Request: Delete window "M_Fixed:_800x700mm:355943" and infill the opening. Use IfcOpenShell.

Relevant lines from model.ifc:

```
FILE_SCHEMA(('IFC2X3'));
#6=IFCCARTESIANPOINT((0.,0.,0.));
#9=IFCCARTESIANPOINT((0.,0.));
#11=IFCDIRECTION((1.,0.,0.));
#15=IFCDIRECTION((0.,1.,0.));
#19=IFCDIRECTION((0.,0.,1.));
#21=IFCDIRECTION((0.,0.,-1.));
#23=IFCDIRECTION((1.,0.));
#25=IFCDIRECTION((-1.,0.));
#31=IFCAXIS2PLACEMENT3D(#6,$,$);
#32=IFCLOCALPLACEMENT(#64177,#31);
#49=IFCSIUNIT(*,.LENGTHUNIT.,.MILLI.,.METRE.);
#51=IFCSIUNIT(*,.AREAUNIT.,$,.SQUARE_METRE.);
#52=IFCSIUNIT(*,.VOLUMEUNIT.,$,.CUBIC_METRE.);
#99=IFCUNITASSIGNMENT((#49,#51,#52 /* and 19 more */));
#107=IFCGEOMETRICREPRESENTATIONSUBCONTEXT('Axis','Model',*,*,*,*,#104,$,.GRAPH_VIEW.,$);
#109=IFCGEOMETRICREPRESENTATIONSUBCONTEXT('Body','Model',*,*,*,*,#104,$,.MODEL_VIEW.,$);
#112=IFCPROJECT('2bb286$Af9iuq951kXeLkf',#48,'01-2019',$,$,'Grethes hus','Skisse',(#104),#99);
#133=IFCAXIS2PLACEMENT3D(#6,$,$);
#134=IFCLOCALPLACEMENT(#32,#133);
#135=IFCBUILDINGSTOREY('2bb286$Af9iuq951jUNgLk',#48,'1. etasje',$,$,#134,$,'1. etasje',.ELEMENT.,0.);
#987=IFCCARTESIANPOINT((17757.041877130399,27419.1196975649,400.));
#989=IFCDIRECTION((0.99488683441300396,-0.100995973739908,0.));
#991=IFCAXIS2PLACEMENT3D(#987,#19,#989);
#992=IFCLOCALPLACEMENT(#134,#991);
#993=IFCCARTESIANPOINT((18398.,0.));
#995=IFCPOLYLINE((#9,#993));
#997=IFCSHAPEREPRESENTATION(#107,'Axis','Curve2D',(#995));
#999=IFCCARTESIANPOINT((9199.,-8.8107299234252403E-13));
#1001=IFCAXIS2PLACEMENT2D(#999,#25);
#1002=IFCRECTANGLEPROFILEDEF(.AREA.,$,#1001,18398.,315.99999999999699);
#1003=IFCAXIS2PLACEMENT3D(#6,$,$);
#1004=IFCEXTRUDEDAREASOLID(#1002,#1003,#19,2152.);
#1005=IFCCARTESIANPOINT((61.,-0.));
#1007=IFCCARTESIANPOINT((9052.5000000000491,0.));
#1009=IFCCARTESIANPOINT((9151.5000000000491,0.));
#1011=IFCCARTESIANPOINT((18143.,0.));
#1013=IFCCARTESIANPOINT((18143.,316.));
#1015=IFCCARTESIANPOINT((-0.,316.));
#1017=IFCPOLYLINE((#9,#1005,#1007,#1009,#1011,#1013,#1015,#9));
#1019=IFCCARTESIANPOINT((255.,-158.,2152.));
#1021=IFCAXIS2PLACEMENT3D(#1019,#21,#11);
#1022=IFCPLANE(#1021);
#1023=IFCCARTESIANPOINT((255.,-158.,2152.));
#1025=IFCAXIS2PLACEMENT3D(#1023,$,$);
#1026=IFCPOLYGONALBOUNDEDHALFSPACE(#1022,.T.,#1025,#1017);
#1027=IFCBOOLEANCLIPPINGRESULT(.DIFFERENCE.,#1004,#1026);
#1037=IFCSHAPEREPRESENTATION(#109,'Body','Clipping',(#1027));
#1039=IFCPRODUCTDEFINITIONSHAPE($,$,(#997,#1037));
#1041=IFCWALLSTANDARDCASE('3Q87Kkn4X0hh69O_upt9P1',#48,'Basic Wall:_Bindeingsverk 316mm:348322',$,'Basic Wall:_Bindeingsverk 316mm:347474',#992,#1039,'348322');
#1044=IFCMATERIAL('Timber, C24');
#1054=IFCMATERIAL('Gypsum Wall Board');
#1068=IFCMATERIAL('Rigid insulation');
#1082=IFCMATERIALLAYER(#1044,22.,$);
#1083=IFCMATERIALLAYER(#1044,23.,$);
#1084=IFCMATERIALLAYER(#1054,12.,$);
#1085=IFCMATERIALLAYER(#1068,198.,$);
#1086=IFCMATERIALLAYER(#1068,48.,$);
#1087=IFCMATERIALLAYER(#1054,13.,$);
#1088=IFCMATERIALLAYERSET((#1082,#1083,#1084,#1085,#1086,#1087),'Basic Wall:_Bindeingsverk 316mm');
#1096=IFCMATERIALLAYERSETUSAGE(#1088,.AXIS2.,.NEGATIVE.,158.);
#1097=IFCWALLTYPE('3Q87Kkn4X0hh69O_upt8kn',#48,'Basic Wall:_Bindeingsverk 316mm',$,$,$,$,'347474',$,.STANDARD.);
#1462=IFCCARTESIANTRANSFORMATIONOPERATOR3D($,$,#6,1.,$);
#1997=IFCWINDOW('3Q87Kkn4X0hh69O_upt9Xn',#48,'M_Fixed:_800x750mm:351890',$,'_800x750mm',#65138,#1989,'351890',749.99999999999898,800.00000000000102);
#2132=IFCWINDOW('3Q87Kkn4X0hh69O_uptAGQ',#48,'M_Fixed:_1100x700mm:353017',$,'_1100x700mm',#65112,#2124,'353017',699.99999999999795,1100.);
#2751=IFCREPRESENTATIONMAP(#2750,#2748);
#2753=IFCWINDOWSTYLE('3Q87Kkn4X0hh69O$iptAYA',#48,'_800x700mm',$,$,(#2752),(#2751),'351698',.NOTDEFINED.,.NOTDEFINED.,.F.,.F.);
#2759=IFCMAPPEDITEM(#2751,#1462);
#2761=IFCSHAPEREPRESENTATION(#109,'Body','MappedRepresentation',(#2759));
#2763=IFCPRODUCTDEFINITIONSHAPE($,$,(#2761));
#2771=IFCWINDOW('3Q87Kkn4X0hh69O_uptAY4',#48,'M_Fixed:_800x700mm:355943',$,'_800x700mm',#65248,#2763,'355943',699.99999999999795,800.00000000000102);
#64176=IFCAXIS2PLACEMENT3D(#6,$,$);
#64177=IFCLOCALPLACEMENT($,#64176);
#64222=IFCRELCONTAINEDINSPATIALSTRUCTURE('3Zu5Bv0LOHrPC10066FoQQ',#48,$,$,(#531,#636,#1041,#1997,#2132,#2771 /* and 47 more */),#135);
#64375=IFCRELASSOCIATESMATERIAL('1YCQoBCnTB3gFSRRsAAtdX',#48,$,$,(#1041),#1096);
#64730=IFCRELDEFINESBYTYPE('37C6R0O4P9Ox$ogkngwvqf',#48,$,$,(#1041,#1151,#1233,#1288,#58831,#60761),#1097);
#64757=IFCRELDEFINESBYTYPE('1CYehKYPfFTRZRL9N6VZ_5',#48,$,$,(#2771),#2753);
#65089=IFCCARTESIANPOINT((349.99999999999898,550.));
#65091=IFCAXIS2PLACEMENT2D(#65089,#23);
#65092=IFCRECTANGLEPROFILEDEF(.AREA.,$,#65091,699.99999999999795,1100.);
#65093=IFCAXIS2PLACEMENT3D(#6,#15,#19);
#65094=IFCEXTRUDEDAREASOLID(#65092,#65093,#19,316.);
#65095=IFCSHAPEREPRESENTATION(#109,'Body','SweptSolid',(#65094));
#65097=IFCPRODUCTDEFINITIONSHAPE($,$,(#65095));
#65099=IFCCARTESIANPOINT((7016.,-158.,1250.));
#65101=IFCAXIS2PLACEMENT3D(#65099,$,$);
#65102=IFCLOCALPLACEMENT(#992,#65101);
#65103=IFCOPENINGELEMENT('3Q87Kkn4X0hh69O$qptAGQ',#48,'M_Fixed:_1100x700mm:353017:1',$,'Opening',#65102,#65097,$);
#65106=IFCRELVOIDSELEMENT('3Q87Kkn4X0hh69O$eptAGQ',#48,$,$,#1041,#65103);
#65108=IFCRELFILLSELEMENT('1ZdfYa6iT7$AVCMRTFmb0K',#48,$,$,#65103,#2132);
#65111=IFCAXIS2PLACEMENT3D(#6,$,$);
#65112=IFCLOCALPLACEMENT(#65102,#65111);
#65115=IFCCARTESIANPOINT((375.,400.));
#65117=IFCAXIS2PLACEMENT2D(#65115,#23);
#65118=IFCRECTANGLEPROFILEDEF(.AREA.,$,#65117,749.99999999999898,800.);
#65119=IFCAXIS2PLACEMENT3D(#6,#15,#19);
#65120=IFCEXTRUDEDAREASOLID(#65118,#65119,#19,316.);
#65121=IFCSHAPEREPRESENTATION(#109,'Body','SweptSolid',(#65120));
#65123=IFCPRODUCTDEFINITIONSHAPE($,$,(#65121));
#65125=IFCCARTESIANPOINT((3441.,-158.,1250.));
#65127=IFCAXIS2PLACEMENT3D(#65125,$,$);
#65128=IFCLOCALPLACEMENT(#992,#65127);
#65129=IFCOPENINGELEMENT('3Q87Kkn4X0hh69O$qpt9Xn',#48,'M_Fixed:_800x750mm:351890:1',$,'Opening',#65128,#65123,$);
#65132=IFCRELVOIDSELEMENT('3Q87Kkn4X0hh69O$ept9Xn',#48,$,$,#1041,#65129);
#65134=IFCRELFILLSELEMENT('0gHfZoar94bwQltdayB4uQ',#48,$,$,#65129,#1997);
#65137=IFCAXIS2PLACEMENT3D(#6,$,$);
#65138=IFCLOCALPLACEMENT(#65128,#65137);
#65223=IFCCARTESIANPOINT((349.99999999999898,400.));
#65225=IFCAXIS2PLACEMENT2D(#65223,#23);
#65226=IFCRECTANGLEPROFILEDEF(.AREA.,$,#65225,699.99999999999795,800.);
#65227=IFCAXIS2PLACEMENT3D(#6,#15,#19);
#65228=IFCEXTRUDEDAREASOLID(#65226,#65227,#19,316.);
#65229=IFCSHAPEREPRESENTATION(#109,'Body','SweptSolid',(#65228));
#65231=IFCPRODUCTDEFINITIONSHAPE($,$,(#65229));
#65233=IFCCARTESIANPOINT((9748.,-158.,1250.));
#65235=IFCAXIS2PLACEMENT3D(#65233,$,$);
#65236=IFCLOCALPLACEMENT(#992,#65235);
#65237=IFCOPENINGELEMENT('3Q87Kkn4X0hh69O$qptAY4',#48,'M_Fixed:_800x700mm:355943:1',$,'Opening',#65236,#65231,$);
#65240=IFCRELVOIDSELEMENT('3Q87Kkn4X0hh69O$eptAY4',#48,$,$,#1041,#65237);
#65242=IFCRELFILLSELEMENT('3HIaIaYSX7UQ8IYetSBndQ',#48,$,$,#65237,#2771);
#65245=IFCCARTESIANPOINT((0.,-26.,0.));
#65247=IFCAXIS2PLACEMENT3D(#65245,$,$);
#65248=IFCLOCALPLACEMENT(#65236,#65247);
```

```python
import ifcopenshell
import ifcopenshell.api.feature
import ifcopenshell.api.root
import ifcopenshell.geom
import ifcopenshell.util.shape

model = ifcopenshell.open("model.ifc")
settings = ifcopenshell.geom.settings()


def volume(element):
    """Net volume in cubic metres, openings subtracted."""
    shape = ifcopenshell.geom.create_shape(settings, element)
    return ifcopenshell.util.shape.get_volume(shape.geometry)


window = model.by_guid("3Q87Kkn4X0hh69O_uptAY4")
opening = window.FillsVoids[0].RelatingOpeningElement
wall = opening.VoidsElements[0].RelatingBuildingElement
before = volume(wall)

ifcopenshell.api.root.remove_product(model, product=window)
ifcopenshell.api.feature.remove_feature(model, feature=opening)

after = volume(wall)

print(f"wall volume {before:.3f} -> {after:.3f} m3")

model.write("model-out.ifc")
```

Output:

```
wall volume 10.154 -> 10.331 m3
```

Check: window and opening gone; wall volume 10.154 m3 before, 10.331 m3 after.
